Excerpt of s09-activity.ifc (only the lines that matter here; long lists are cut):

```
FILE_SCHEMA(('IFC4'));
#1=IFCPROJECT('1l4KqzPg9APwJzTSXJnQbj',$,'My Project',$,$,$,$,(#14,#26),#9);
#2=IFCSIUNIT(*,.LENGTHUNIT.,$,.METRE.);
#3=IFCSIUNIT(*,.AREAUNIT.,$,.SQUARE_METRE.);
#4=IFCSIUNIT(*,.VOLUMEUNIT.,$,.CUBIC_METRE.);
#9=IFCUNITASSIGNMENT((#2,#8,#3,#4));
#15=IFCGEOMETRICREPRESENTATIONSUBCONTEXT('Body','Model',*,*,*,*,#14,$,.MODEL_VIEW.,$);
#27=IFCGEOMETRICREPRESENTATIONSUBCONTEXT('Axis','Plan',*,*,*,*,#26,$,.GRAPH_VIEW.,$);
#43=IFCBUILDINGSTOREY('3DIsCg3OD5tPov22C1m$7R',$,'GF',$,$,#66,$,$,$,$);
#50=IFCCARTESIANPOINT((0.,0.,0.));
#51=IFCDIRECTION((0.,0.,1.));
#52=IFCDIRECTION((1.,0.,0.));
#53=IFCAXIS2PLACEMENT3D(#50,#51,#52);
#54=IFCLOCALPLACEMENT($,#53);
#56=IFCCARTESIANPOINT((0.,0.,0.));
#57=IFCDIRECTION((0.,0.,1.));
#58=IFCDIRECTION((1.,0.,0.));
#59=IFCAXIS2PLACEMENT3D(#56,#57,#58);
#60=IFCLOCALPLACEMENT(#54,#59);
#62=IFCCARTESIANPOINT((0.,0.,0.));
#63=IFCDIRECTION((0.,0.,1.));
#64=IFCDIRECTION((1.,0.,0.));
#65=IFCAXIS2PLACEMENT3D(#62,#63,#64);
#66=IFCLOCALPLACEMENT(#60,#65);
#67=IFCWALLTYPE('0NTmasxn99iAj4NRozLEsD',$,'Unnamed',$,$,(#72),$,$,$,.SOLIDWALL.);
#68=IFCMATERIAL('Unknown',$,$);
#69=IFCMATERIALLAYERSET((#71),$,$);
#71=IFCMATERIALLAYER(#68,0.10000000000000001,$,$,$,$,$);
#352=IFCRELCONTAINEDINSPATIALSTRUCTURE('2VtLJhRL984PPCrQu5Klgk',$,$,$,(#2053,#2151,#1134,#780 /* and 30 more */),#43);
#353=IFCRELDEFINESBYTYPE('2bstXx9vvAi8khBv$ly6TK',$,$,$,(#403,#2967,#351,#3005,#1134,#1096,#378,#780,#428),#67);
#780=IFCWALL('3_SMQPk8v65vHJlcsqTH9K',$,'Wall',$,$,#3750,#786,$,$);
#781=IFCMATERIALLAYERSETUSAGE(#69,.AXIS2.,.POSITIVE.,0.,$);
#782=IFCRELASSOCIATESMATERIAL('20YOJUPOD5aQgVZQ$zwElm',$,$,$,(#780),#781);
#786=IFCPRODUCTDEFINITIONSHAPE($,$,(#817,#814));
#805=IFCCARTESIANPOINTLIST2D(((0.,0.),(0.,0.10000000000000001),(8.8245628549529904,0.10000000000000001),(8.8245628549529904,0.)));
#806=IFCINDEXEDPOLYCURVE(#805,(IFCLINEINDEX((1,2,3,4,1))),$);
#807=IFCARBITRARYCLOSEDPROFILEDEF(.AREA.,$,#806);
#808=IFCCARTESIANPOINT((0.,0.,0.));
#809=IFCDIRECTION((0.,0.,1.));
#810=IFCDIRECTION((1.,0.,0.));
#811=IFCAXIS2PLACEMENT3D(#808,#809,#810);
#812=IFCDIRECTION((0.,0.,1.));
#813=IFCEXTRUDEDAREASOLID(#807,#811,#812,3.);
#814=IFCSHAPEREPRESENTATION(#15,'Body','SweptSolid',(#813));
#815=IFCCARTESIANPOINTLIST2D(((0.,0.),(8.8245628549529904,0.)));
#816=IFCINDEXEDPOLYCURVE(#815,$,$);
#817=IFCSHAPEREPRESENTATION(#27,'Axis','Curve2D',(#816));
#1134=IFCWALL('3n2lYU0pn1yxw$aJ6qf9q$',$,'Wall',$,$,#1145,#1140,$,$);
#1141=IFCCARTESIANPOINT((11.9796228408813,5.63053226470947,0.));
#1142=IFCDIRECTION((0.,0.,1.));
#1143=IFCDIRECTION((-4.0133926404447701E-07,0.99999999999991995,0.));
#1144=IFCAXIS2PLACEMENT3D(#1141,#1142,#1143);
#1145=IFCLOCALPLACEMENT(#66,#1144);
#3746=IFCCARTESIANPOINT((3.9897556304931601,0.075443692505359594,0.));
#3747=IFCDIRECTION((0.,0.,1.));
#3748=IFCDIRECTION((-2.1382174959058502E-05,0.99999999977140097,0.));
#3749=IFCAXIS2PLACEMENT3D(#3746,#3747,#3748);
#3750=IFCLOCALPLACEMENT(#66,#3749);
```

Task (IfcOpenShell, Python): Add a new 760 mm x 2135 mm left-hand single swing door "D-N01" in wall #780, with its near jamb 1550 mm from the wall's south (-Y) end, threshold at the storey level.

```python
import numpy as np
import ifcopenshell
import ifcopenshell.api.feature
import ifcopenshell.api.geometry
import ifcopenshell.api.root
import ifcopenshell.api.spatial
import ifcopenshell.geom
import ifcopenshell.util.element
import ifcopenshell.util.placement
import ifcopenshell.util.representation
import ifcopenshell.util.shape
import ifcopenshell.util.unit

model = ifcopenshell.open("s09-activity.ifc")
unit_scale = ifcopenshell.util.unit.calculate_unit_scale(model)
settings = ifcopenshell.geom.settings()


def volume(element):
    """Net volume in cubic metres, openings subtracted."""
    shape = ifcopenshell.geom.create_shape(settings, element)
    return ifcopenshell.util.shape.get_volume(shape.geometry)


wall = model.by_guid("3_SMQPk8v65vHJlcsqTH9K")
storey = ifcopenshell.util.element.get_container(wall, ifc_class="IfcBuildingStorey")
context = ifcopenshell.util.representation.get_context(model, "Model", "Body", "MODEL_VIEW")
before = volume(wall)

width, height, from_end, sill = 0.76, 2.135, 1.55, 0.0  # metres

# The wall runs along its own X axis, and the end named is its -X end.
wall_shape = ifcopenshell.geom.create_shape(settings, wall)
x, y, z = ifcopenshell.util.shape.get_vertices(wall_shape.geometry).T
start = x.min() + from_end
face, thickness = float(y.min()), float(y.max() - y.min())
wall_matrix = ifcopenshell.util.placement.get_local_placement(wall.ObjectPlacement)
level = ifcopenshell.util.placement.get_local_placement(storey.ObjectPlacement)[2, 3]


def in_wall(x, y):
    """Placement at x, y metres in the wall's axes, at sill height."""
    matrix = wall_matrix.copy()
    matrix[:, 3] = wall_matrix @ np.array([x / unit_scale, y / unit_scale, 0.0, 1.0])
    matrix[2, 3] = level + sill / unit_scale
    return matrix


# Opening: a box that overshoots both wall faces by 50 mm.
opening = ifcopenshell.api.root.create_entity(model, ifc_class="IfcOpeningElement", predefined_type="OPENING")
box = ifcopenshell.api.geometry.add_wall_representation(
    model, context=context, length=width, height=height, thickness=thickness + 0.1
)
ifcopenshell.api.geometry.assign_representation(model, product=opening, representation=box)
ifcopenshell.api.geometry.edit_object_placement(model, product=opening, matrix=in_wall(start, face - 0.05), is_si=False)
ifcopenshell.api.feature.add_feature(model, feature=opening, element=wall)

door = ifcopenshell.api.root.create_entity(model, ifc_class="IfcDoor", name="D-N01", predefined_type="DOOR")
door.OverallWidth, door.OverallHeight = width / unit_scale, height / unit_scale
door.OperationType = "SINGLE_SWING_LEFT"
body = ifcopenshell.api.geometry.add_door_representation(
    model,
    context=context,
    overall_width=door.OverallWidth,
    overall_height=door.OverallHeight,
    operation_type="SINGLE_SWING_LEFT",
    lining_properties={"LiningDepth": thickness / unit_scale, "ThresholdDepth": thickness / unit_scale},
)
ifcopenshell.api.geometry.assign_representation(model, product=door, representation=body)
ifcopenshell.api.spatial.assign_container(model, products=[door], relating_structure=storey)
ifcopenshell.api.feature.add_filling(model, opening=opening, element=door)

# The lining spans the wall, so the door starts at the wall face.
ifcopenshell.api.geometry.edit_object_placement(model, product=door, matrix=in_wall(start, face), is_si=False)

after = volume(wall)

print(f"wall volume {before:.3f} -> {after:.3f} m3")

model.write("s09-activity_v2.ifc")
```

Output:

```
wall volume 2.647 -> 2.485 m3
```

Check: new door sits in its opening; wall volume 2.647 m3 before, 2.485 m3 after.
